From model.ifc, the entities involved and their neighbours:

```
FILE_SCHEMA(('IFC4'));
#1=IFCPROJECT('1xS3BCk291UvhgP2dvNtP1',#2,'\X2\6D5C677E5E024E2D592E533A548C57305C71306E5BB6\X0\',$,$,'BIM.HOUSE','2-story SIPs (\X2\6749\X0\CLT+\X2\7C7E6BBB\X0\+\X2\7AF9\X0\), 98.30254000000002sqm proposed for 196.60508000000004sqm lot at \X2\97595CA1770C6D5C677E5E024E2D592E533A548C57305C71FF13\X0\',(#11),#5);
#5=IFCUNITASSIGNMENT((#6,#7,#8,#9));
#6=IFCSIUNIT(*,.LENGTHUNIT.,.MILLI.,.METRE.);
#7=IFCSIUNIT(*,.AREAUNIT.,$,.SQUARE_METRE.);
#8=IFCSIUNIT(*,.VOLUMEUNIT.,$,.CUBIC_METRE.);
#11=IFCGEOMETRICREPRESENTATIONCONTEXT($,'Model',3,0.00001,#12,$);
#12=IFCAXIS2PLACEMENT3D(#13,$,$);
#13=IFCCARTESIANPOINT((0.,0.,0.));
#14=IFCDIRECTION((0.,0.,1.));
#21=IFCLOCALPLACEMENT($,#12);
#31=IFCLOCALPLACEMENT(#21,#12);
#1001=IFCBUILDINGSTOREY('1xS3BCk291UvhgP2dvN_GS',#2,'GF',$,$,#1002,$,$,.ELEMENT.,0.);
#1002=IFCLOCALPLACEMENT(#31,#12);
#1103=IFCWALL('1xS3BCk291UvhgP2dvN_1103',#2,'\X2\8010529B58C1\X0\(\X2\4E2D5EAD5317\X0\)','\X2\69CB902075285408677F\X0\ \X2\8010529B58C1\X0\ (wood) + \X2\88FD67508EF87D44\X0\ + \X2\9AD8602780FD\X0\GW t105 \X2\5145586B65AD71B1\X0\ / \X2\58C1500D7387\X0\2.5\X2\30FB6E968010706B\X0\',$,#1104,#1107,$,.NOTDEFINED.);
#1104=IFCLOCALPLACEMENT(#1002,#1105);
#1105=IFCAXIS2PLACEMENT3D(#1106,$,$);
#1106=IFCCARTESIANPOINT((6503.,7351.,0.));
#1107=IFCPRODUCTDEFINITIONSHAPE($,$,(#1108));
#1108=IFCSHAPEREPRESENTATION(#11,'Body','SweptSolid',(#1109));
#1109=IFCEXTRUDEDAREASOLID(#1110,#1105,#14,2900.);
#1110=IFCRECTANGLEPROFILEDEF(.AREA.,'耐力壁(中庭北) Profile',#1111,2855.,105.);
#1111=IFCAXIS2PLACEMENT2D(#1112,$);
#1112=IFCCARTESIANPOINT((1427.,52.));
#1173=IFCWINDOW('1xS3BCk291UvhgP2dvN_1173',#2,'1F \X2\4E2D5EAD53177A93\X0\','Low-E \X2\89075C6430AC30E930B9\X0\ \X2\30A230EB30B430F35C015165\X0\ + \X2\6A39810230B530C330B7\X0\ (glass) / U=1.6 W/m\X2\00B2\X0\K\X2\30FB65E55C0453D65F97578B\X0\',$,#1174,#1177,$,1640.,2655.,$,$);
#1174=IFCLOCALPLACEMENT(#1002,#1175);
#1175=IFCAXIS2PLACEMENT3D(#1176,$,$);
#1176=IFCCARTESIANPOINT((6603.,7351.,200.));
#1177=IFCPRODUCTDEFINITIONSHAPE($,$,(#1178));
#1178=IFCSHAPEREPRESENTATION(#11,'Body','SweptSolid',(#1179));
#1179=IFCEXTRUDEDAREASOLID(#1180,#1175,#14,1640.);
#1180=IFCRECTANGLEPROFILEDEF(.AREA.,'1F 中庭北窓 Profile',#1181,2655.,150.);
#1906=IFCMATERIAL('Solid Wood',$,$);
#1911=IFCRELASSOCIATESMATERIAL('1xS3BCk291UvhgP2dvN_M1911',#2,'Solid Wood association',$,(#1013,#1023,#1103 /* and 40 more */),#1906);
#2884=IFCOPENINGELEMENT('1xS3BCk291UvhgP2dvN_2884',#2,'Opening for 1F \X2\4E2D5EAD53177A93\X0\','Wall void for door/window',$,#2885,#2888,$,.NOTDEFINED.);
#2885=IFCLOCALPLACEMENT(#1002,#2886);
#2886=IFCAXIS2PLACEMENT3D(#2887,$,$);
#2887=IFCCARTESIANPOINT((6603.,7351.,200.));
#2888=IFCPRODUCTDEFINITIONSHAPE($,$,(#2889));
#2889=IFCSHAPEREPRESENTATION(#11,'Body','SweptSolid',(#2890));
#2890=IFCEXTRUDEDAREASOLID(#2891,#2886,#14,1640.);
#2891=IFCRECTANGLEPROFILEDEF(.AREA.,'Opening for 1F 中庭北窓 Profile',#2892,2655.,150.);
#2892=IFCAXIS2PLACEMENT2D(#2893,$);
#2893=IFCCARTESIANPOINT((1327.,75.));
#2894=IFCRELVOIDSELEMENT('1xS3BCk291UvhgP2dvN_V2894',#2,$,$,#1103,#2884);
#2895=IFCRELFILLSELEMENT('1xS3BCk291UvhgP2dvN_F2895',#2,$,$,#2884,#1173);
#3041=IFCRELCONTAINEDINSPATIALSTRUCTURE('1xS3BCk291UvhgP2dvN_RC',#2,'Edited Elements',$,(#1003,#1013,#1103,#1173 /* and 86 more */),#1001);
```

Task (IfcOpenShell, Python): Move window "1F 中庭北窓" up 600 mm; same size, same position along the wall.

```python
import numpy as np
import ifcopenshell
import ifcopenshell.api.geometry
import ifcopenshell.util.placement
import ifcopenshell.util.unit

model = ifcopenshell.open("model.ifc")
unit_scale = ifcopenshell.util.unit.calculate_unit_scale(model)

window = model.by_guid("1xS3BCk291UvhgP2dvN_1173")
opening = window.FillsVoids[0].RelatingOpeningElement
dz = 0.6 / unit_scale

shift = np.array([0.0, 0.0, dz])
# The window is not placed relative to its opening, so move both.
for product in (opening, window):
    matrix = ifcopenshell.util.placement.get_local_placement(product.ObjectPlacement)
    matrix[:3, 3] += shift
    ifcopenshell.api.geometry.edit_object_placement(model, product=product, matrix=matrix, is_si=False)

print(f"moved by {dz * unit_scale:+.3f} m")

model.write("model_rev.ifc")
```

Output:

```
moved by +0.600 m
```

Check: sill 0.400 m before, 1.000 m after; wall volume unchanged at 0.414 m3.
